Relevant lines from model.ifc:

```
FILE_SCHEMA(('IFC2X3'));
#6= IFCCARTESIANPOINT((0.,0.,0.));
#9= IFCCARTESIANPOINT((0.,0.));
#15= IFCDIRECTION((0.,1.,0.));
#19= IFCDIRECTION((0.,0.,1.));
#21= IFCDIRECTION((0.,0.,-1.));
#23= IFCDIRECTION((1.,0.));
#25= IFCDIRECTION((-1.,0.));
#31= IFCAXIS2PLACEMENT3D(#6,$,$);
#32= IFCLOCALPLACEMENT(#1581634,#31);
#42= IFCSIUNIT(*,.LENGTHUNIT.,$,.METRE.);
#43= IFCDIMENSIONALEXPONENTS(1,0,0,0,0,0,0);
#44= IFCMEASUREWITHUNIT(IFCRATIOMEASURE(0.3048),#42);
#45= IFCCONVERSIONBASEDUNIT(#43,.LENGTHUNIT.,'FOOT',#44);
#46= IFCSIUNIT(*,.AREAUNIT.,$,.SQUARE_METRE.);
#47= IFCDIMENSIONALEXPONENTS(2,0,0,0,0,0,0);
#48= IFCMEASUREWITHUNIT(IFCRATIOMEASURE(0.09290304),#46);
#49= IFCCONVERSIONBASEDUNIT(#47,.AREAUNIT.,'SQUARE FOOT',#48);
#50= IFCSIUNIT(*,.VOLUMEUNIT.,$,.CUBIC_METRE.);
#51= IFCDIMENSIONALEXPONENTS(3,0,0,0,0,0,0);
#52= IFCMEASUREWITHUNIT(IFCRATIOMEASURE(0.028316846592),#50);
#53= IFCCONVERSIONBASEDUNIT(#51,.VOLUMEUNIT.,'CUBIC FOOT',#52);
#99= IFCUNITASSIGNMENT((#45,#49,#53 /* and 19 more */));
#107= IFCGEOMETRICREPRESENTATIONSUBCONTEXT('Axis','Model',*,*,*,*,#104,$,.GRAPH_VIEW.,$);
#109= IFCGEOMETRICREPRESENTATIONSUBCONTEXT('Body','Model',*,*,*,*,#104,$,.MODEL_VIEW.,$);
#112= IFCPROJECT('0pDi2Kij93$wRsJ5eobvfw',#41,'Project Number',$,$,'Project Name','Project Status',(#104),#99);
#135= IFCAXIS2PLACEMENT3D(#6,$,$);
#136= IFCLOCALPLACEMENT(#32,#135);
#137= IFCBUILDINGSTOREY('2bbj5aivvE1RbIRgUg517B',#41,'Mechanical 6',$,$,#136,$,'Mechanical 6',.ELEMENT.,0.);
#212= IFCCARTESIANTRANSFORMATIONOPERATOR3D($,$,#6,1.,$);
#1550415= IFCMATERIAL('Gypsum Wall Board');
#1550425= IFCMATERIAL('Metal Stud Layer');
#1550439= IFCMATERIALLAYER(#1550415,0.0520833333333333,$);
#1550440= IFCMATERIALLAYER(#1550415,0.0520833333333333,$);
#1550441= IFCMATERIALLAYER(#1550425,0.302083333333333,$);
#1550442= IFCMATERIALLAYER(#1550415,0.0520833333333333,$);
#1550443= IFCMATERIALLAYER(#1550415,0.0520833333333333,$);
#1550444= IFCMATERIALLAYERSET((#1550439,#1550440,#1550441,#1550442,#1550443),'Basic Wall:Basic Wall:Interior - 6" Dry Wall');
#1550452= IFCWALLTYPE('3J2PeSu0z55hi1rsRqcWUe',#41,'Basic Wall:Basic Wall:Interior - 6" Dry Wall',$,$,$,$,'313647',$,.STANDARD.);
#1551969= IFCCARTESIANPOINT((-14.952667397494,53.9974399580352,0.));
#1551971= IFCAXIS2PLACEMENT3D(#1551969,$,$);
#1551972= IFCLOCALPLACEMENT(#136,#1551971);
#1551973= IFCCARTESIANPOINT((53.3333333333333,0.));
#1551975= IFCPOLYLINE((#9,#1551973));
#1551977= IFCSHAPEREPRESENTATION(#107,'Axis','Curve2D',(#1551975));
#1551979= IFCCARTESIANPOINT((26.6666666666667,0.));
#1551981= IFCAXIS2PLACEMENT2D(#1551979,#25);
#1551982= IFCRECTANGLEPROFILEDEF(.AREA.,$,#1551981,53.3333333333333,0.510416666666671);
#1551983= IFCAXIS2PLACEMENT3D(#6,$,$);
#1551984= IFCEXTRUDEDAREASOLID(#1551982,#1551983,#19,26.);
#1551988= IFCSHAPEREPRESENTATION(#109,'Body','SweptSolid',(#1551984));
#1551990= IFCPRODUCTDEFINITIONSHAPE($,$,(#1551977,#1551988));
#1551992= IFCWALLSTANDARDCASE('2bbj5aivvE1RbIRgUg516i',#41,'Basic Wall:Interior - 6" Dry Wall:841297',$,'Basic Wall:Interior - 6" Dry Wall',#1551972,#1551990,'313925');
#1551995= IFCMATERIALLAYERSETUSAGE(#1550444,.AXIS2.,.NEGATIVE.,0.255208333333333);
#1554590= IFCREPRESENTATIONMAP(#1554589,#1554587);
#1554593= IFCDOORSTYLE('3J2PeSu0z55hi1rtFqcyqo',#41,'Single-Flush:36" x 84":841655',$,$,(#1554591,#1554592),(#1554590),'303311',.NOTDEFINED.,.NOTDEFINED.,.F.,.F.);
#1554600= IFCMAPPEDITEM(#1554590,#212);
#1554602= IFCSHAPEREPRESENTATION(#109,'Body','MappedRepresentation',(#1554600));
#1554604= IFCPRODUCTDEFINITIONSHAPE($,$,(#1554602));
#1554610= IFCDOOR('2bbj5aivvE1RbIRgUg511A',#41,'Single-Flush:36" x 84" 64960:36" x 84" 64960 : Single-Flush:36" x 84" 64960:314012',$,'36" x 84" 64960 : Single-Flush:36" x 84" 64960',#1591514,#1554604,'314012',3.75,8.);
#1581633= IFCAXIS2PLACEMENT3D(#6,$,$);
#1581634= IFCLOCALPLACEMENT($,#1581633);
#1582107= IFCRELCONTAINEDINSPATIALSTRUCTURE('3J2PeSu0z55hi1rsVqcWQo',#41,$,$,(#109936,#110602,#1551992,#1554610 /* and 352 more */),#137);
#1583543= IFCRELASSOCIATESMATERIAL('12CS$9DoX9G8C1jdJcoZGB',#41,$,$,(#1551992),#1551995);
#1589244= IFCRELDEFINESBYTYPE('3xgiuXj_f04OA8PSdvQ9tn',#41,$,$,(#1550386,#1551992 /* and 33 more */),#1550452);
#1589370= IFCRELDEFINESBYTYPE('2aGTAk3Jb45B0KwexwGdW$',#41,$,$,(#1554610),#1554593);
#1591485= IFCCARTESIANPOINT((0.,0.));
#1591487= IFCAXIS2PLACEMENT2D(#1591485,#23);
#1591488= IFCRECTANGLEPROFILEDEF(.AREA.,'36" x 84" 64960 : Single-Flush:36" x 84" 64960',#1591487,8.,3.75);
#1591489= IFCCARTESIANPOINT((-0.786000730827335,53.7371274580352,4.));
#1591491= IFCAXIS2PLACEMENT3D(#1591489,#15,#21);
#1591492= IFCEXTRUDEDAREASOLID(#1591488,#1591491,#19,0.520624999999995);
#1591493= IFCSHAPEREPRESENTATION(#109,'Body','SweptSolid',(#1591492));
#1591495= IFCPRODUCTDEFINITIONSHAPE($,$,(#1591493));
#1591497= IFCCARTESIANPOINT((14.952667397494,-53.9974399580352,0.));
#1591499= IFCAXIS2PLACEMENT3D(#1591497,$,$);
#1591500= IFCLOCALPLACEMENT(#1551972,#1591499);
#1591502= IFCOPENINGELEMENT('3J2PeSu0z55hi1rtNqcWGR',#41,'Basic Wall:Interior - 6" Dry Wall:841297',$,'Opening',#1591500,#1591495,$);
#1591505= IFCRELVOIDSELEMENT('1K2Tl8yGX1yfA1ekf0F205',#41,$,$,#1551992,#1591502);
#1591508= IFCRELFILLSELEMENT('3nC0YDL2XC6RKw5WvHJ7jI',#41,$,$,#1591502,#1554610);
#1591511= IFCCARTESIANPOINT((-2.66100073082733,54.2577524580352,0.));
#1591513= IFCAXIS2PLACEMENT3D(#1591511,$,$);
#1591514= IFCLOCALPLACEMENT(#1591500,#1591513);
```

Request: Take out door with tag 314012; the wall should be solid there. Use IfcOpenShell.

```python
import ifcopenshell
import ifcopenshell.api.feature
import ifcopenshell.api.root
import ifcopenshell.geom
import ifcopenshell.util.shape

model = ifcopenshell.open("model.ifc")
settings = ifcopenshell.geom.settings()


def volume(element):
    """Net volume in cubic metres, openings subtracted."""
    shape = ifcopenshell.geom.create_shape(settings, element)
    return ifcopenshell.util.shape.get_volume(shape.geometry)


door = model.by_id(1554610)
opening = door.FillsVoids[0].RelatingOpeningElement
wall = opening.VoidsElements[0].RelatingBuildingElement
before = volume(wall)

ifcopenshell.api.root.remove_product(model, product=door)
ifcopenshell.api.feature.remove_feature(model, feature=opening)

after = volume(wall)

print(f"wall volume {before:.3f} -> {after:.3f} m3")

model.write("model_edited.ifc")
```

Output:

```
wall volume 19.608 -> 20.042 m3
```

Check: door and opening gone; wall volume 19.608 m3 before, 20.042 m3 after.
